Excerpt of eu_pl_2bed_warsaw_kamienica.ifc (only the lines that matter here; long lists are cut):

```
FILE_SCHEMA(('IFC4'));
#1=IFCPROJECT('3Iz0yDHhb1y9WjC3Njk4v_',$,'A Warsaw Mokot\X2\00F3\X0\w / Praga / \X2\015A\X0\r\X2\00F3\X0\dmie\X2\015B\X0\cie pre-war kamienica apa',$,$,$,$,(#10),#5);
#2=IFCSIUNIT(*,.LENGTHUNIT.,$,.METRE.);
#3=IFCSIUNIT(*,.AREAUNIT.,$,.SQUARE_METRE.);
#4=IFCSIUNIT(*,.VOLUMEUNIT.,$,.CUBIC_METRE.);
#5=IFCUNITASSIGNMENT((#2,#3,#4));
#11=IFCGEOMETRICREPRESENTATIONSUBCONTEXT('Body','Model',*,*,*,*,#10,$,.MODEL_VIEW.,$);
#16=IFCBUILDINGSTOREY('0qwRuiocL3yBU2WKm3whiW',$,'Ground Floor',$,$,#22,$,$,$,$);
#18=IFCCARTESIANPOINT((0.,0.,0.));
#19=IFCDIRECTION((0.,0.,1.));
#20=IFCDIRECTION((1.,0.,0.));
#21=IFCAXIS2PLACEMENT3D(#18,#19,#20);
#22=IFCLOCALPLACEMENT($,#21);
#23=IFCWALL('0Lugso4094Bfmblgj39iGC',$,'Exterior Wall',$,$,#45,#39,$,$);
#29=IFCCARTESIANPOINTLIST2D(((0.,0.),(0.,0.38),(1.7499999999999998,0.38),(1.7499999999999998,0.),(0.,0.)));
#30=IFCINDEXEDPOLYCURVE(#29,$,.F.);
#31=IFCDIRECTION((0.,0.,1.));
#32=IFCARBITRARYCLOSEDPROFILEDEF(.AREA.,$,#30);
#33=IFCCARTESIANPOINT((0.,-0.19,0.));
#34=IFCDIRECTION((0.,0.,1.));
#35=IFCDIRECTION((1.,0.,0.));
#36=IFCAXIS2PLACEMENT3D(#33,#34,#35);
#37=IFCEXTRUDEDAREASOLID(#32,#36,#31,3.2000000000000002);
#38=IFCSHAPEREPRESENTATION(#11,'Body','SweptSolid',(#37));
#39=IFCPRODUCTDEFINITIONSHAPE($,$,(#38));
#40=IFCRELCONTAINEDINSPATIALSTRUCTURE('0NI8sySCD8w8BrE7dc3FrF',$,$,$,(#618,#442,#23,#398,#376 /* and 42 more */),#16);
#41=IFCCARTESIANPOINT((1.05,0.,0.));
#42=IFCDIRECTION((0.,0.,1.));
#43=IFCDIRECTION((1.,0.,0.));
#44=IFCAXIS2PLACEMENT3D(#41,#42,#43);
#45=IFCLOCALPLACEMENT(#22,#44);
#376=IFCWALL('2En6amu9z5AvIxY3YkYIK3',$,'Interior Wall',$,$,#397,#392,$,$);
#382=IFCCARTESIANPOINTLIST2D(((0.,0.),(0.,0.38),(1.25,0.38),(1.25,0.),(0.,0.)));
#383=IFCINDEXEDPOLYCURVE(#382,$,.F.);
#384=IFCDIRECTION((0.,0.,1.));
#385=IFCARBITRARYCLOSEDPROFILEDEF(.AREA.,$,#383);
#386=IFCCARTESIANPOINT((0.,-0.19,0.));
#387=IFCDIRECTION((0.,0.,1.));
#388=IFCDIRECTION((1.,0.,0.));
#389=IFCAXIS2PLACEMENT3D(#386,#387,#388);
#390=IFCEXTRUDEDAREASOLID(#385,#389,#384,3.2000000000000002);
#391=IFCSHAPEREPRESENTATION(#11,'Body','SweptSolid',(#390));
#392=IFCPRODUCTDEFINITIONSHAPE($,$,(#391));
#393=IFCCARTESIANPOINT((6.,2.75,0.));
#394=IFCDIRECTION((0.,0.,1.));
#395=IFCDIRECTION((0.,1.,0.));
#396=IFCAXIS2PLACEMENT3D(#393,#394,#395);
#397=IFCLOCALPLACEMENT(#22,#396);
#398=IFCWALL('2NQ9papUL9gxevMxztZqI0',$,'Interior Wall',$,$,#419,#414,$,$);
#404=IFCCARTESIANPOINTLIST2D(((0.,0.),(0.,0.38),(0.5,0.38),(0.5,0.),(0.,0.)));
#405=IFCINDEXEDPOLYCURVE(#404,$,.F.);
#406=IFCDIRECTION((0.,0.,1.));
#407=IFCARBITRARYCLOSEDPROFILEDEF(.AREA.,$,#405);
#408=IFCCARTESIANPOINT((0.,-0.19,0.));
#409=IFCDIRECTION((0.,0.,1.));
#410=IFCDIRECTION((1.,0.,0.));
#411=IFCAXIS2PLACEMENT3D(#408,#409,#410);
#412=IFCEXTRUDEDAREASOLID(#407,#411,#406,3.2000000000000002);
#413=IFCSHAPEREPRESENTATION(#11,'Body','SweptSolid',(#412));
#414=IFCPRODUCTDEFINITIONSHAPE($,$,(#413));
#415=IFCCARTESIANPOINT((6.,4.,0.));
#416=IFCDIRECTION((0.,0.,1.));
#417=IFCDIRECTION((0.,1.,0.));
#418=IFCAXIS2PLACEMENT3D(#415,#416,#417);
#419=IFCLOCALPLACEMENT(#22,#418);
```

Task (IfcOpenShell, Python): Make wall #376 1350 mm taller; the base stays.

```python
import ifcopenshell
import ifcopenshell.geom
import ifcopenshell.util.representation
import ifcopenshell.util.shape
import ifcopenshell.util.unit

model = ifcopenshell.open("eu_pl_2bed_warsaw_kamienica.ifc")
unit_scale = ifcopenshell.util.unit.calculate_unit_scale(model)
settings = ifcopenshell.geom.settings()


def volume(element):
    """Net volume in cubic metres, openings subtracted."""
    shape = ifcopenshell.geom.create_shape(settings, element)
    return ifcopenshell.util.shape.get_volume(shape.geometry)


wall = model.by_id(376)
before = volume(wall)

body = ifcopenshell.util.representation.get_representation(wall, "Model", "Body")
solid = body.Items[0]
old_height = solid.Depth
solid.Depth += 1.35 / unit_scale
after = volume(wall)

print(f"height {old_height:g} -> {solid.Depth:g}, volume {before:.3f} -> {after:.3f} m3")

model.write("eu_pl_2bed_warsaw_kamienica_rev.ifc")
```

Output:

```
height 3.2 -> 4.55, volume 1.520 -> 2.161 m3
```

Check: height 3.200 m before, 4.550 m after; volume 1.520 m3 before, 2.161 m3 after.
